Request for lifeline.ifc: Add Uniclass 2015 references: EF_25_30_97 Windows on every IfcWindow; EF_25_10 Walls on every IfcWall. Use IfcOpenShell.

First a look at what the model holds.

```python
import ifcopenshell

model = ifcopenshell.open("lifeline.ifc")
print(model.schema)
print("classifications:", [c.Name for c in model.by_type("IfcClassification")])
for ifc_class in ("IfcDoor", "IfcRoof", "IfcStair", "IfcWall", "IfcWindow"):
    print(ifc_class, len(model.by_type(ifc_class)))
```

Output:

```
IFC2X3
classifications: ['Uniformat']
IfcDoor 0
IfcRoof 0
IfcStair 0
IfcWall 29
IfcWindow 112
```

```python
import ifcopenshell
import ifcopenshell.api.classification

model = ifcopenshell.open("lifeline.ifc")

# IFC2X3 requires Source and Edition and has no link from the project to the system.
system = model.create_entity("IfcClassification", Source="NBS", Edition="2015", Name="Uniclass 2015")

codes = {
    "IfcWindow": ("EF_25_30_97", "Windows"),
    "IfcWall": ("EF_25_10", "Walls"),
}
for ifc_class, (code, name) in codes.items():
    products = model.by_type(ifc_class)
    ifcopenshell.api.classification.add_reference(
        model, products=products, classification=system, identification=code, name=name
    )
    print(code, len(products))

model.write("lifeline_updated.ifc")
```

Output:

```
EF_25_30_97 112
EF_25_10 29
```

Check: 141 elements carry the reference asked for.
